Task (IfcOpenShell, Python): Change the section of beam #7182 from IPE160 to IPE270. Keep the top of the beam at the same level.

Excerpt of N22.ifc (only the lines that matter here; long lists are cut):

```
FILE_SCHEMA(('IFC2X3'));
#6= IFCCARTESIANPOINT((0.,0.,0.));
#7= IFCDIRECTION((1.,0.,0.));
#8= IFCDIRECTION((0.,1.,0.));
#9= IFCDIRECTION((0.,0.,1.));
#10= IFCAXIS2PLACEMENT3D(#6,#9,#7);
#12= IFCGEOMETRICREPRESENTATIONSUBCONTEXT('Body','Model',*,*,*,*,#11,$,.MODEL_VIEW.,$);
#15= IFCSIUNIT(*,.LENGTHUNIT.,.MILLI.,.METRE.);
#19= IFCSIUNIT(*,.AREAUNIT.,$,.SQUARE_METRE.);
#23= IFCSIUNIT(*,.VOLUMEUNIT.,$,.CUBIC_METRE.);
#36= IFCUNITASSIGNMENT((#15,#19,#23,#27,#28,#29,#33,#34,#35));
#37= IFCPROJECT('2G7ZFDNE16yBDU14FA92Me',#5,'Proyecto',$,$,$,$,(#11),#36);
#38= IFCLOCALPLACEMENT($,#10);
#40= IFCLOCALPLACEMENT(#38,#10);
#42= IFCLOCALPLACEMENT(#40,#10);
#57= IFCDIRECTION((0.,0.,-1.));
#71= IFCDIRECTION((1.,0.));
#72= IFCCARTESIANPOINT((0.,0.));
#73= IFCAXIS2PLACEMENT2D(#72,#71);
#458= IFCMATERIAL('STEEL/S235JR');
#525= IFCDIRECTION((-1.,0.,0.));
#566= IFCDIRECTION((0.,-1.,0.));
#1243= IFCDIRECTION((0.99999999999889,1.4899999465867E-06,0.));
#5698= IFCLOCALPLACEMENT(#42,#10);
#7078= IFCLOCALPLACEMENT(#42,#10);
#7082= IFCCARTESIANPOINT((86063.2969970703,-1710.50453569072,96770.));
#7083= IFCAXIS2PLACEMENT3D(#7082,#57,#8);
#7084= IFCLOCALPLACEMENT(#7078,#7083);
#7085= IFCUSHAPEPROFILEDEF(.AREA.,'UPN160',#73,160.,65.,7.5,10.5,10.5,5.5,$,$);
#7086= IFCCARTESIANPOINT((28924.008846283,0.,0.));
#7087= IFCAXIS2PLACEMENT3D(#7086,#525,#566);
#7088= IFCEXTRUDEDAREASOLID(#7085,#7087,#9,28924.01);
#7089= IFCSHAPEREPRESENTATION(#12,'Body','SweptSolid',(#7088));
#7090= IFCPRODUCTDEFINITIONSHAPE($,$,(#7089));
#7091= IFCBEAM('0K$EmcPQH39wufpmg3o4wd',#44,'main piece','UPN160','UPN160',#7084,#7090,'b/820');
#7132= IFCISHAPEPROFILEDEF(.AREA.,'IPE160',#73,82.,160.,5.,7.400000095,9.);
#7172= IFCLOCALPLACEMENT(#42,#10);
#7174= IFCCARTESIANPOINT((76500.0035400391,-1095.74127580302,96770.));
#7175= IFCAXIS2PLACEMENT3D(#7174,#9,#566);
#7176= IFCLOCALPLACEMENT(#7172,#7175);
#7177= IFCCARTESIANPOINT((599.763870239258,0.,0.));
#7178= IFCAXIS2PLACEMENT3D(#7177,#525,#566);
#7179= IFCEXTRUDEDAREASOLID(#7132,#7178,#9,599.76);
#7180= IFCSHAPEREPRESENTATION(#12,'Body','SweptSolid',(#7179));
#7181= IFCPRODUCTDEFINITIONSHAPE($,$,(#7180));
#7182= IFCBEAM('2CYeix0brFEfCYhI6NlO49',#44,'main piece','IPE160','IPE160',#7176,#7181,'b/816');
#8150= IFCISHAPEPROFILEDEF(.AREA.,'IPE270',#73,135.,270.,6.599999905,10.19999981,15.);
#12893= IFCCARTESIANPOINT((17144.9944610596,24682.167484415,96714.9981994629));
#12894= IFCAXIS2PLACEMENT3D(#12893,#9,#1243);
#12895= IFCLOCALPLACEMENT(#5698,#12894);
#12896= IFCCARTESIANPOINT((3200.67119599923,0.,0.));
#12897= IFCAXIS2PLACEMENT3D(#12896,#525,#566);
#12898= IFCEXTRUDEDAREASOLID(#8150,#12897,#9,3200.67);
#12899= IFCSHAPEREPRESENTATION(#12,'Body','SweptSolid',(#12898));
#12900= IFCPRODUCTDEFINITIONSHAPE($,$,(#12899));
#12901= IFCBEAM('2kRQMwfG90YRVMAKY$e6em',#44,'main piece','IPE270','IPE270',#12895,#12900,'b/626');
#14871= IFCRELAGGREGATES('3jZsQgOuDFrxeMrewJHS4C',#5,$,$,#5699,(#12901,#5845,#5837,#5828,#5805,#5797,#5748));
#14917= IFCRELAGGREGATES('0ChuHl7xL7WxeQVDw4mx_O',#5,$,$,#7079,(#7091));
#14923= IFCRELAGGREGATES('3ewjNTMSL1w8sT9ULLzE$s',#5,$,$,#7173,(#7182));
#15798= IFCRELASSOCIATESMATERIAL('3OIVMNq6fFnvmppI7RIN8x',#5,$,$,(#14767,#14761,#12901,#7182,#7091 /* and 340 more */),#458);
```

```python
import ifcopenshell
import ifcopenshell.util.element
import ifcopenshell.util.representation

model = ifcopenshell.open("N22.ifc")

member = model.by_guid("2CYeix0brFEfCYhI6NlO49")
source = next(p for p in model.by_type("IfcIShapeProfileDef") if p.ProfileName == "IPE270")

body = ifcopenshell.util.representation.get_representation(member, "Model", "Body")
solid = body.Items[0]
old_profile = solid.SweptArea

# Copy the section's sizes but keep this member's own profile position.
profile = ifcopenshell.util.element.copy(model, source)
# Profiles are centred, so shift by half the change in depth to hold the top.
shift = (old_profile.OverallDepth - profile.OverallDepth) / 2
x, y = old_profile.Position.Location.Coordinates
up = (0.0, 1.0)  # upwards, in the solid's own plane
location = model.createIfcCartesianPoint((x + up[0] * shift, y + up[1] * shift))
profile.Position = model.createIfcAxis2Placement2D(location, old_profile.Position.RefDirection)
solid.SweptArea = profile
if not model.get_total_inverses(old_profile):
    ifcopenshell.util.element.remove_deep2(model, old_profile)
member.Description = member.Description.replace("IPE160", "IPE270")
member.ObjectType = member.ObjectType.replace("IPE160", "IPE270")

print(solid.SweptArea)

model.write("N22_v2.ifc")
```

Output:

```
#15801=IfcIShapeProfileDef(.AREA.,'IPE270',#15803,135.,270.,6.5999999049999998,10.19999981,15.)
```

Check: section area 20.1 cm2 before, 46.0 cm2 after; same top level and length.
